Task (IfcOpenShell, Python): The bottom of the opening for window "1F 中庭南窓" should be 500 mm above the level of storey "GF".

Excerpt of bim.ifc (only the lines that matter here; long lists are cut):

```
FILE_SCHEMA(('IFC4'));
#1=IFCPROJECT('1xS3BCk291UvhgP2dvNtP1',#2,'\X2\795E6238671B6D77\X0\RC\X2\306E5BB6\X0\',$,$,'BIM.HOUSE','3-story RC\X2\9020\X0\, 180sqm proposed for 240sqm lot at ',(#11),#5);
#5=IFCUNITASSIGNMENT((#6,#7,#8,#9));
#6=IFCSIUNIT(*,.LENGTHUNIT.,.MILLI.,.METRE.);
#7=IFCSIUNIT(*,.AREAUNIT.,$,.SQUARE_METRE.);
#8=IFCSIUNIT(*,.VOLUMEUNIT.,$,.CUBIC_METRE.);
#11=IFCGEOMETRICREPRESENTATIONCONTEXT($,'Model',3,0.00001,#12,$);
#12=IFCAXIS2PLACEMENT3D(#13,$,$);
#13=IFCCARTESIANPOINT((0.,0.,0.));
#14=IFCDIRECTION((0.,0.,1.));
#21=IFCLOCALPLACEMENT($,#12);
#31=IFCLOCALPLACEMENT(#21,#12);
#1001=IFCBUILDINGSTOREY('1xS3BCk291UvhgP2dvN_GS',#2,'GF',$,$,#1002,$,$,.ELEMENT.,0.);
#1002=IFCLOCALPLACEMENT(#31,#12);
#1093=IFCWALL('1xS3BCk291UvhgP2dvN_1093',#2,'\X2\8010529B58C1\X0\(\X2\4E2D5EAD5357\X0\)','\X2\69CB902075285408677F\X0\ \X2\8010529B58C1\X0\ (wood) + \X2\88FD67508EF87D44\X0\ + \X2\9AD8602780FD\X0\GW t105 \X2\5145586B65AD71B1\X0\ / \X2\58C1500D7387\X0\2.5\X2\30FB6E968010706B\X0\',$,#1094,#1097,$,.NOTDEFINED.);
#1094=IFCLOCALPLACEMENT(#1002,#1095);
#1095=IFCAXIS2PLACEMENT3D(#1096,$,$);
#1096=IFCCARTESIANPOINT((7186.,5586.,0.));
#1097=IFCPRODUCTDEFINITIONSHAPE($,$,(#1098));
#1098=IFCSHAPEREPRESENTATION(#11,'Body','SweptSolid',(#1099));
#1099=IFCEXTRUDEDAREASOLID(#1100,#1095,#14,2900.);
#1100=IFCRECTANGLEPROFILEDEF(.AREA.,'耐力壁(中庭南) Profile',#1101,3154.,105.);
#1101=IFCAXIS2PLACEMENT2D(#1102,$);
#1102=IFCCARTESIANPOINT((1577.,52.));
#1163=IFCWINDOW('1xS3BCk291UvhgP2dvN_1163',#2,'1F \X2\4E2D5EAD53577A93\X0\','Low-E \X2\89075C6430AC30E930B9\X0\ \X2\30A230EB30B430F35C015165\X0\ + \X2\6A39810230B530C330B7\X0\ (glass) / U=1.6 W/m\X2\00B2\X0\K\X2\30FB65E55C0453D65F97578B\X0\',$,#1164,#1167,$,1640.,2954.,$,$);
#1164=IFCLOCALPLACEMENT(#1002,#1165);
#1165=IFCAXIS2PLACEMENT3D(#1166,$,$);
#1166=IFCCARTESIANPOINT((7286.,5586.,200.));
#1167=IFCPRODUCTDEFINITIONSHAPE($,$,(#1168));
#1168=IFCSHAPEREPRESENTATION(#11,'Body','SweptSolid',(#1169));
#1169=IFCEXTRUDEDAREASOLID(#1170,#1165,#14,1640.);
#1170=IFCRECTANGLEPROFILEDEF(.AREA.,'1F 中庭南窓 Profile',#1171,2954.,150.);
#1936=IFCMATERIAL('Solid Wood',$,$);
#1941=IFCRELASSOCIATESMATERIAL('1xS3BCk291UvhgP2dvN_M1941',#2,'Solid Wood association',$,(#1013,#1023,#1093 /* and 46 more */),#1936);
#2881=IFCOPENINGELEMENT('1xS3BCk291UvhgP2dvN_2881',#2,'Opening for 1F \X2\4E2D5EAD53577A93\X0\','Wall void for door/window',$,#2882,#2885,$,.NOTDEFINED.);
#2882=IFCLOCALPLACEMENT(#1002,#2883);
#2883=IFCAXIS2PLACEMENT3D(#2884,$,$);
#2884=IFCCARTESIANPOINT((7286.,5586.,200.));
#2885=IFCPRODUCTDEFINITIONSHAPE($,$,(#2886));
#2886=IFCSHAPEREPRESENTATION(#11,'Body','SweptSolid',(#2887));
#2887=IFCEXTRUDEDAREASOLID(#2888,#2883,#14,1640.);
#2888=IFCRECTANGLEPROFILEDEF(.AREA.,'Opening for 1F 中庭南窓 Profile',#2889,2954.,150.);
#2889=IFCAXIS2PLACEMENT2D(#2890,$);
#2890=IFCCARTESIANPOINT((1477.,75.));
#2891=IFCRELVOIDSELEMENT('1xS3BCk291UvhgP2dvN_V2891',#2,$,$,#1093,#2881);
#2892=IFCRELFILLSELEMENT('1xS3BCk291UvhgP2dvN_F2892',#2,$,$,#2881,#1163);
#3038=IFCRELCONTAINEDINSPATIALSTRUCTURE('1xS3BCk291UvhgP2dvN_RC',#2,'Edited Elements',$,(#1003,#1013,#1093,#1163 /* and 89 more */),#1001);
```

```python
import numpy as np
import ifcopenshell
import ifcopenshell.api.geometry
import ifcopenshell.geom
import ifcopenshell.util.element
import ifcopenshell.util.placement
import ifcopenshell.util.shape
import ifcopenshell.util.unit

model = ifcopenshell.open("bim.ifc")
unit_scale = ifcopenshell.util.unit.calculate_unit_scale(model)

window = model.by_guid("1xS3BCk291UvhgP2dvN_1163")
opening = window.FillsVoids[0].RelatingOpeningElement
storey = ifcopenshell.util.element.get_container(window, ifc_class="IfcBuildingStorey")
level = ifcopenshell.util.placement.get_local_placement(storey.ObjectPlacement)[2, 3]

# The opening's origin need not be at the sill, so measure its lowest point.
shape = ifcopenshell.geom.create_shape(ifcopenshell.geom.settings(), opening)
bottom = ifcopenshell.util.shape.get_shape_bottom_elevation(shape, shape.geometry) / unit_scale
dz = level + 0.5 / unit_scale - bottom

shift = np.array([0.0, 0.0, dz])
# The window is not placed relative to its opening, so move both.
for product in (opening, window):
    matrix = ifcopenshell.util.placement.get_local_placement(product.ObjectPlacement)
    matrix[:3, 3] += shift
    ifcopenshell.api.geometry.edit_object_placement(model, product=product, matrix=matrix, is_si=False)

print(f"moved by {dz * unit_scale:+.3f} m")

model.write("bim-out.ifc")
```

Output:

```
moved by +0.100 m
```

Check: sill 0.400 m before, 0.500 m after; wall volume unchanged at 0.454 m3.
